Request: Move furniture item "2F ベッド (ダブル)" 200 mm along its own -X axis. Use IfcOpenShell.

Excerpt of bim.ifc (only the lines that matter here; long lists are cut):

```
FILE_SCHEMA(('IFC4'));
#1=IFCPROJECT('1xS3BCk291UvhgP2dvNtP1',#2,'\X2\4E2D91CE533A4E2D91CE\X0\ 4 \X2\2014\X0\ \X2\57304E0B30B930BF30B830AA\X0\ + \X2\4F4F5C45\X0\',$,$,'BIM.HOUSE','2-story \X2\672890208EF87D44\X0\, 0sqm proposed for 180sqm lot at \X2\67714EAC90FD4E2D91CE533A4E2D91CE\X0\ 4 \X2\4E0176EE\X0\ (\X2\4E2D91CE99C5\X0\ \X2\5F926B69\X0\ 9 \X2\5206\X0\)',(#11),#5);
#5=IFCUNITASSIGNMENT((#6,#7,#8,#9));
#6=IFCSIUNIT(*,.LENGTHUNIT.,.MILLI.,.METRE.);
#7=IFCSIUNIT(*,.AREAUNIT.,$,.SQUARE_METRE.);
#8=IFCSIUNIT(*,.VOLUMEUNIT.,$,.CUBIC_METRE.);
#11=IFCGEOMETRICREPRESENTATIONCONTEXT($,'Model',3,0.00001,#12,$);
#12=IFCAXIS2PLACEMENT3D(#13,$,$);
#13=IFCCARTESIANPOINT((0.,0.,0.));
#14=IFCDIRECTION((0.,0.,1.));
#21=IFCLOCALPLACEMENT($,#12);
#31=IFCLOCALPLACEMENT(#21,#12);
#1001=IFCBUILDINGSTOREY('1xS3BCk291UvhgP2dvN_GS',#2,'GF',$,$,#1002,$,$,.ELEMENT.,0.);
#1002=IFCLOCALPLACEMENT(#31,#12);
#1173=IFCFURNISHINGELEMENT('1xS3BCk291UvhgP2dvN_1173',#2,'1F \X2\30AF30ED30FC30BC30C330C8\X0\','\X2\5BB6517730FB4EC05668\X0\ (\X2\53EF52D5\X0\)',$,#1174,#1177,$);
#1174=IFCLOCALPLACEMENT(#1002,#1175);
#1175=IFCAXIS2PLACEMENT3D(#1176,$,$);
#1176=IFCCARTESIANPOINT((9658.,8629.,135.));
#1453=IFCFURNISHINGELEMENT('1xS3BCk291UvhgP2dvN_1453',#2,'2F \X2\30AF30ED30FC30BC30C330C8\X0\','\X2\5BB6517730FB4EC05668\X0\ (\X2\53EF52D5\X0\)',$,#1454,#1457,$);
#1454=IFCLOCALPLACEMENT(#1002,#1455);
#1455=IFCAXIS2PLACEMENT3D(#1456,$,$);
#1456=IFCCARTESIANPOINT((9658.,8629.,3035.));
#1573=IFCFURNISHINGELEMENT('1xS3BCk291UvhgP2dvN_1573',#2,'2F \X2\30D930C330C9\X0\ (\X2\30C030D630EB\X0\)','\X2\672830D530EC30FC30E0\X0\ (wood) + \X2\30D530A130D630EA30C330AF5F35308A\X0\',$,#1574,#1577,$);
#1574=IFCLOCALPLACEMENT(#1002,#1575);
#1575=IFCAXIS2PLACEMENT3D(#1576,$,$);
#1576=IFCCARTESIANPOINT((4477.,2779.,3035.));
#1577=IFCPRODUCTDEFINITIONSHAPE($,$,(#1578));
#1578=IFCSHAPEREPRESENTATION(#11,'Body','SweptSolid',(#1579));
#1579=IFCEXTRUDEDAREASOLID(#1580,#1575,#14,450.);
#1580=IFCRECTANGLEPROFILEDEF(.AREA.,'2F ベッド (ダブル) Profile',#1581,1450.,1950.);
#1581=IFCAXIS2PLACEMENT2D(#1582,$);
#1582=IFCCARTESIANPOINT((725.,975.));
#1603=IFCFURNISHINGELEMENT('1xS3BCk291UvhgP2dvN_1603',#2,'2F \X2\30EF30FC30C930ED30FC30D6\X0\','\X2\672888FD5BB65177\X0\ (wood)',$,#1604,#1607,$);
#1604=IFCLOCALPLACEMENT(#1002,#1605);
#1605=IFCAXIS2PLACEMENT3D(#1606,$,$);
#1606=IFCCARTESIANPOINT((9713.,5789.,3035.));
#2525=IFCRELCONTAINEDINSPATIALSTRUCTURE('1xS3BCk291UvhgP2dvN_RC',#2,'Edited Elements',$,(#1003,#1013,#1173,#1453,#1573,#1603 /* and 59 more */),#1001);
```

```python
import ifcopenshell
import ifcopenshell.api.geometry
import ifcopenshell.util.placement
import ifcopenshell.util.unit

model = ifcopenshell.open("bim.ifc")
unit_scale = ifcopenshell.util.unit.calculate_unit_scale(model)

item = model.by_guid("1xS3BCk291UvhgP2dvN_1573")
matrix = ifcopenshell.util.placement.get_local_placement(item.ObjectPlacement)
matrix[:3, 3] -= matrix[:3, 0] * 0.2 / unit_scale
ifcopenshell.api.geometry.edit_object_placement(model, product=item, matrix=matrix, is_si=False)

print(ifcopenshell.util.placement.get_local_placement(item.ObjectPlacement).round(3) + 0.0)

model.write("bim_v2.ifc")
```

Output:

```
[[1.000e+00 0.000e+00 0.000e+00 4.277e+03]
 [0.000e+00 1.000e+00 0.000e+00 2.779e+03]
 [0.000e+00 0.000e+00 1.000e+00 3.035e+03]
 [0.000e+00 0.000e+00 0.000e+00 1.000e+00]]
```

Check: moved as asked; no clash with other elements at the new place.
